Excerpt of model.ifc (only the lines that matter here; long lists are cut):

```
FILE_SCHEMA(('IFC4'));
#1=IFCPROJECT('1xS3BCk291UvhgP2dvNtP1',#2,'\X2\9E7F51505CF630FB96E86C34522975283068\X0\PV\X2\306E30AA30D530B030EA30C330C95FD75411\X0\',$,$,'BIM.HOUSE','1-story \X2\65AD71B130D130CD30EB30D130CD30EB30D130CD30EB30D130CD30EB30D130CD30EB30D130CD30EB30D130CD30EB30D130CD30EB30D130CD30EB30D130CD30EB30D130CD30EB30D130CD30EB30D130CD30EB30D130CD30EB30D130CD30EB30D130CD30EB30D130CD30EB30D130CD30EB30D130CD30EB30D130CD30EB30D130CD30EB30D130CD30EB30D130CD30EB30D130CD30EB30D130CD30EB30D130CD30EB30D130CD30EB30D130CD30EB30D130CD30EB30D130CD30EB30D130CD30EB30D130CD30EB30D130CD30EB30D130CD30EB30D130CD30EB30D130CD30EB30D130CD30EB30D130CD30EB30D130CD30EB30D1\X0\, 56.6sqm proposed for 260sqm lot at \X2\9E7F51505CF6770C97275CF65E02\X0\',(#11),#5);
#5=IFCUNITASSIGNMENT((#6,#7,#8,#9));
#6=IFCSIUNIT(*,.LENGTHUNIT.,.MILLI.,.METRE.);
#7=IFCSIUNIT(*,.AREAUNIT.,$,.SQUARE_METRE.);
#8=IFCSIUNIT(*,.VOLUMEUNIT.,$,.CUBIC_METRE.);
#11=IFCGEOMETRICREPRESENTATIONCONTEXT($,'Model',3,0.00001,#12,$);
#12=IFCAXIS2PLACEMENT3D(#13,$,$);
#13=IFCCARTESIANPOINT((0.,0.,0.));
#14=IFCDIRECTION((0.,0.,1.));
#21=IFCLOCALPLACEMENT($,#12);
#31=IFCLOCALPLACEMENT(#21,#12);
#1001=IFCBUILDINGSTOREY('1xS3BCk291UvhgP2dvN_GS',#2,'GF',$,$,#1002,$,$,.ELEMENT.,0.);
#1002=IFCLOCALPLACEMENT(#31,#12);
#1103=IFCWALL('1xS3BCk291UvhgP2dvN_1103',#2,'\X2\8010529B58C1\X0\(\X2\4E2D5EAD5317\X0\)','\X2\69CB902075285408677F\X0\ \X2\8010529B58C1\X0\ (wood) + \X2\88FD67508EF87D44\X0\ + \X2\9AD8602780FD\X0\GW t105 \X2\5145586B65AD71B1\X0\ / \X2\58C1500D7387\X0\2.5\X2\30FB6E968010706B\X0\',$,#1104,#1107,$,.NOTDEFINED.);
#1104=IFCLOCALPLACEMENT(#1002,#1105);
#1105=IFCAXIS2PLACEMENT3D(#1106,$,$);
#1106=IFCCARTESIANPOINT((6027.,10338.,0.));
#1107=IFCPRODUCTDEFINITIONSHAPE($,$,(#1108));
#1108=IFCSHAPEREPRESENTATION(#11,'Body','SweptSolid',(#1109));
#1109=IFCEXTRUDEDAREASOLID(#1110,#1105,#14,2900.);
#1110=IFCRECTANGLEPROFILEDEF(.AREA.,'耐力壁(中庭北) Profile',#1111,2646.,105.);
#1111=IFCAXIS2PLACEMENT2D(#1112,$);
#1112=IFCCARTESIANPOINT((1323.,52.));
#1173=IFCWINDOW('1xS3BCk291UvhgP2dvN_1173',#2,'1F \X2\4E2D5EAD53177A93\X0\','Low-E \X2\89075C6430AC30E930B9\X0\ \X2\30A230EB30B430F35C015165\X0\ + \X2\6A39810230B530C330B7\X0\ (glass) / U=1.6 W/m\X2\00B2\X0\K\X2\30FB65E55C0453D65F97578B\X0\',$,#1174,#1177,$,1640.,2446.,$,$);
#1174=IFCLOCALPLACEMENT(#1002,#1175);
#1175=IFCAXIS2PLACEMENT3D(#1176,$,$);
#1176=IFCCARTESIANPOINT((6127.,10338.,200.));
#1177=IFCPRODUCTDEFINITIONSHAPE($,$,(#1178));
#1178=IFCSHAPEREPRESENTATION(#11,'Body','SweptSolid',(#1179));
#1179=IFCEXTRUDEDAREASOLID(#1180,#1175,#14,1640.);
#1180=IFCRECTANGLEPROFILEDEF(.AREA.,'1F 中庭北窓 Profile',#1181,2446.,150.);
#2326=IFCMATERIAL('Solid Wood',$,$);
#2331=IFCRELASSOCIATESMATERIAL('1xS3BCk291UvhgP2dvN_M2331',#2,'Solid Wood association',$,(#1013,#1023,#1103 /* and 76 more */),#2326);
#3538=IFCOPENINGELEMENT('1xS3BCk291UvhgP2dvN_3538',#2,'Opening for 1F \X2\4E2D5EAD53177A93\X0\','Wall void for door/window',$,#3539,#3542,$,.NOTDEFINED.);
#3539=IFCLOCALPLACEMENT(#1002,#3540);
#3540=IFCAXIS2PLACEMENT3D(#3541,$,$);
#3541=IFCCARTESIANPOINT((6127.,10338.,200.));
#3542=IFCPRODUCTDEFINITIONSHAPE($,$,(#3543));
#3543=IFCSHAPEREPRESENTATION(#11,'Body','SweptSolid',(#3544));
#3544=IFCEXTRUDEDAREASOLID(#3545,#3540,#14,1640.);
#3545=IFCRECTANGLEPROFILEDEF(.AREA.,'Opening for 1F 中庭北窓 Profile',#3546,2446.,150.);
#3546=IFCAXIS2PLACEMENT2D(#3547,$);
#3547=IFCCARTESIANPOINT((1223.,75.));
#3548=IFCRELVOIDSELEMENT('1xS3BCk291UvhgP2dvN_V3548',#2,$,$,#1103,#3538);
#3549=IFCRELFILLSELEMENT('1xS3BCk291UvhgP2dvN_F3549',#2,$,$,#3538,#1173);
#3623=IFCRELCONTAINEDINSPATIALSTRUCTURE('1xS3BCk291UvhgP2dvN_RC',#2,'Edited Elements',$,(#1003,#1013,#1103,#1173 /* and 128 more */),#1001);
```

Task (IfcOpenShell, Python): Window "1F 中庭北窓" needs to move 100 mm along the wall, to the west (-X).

```python
import ifcopenshell
import ifcopenshell.api.geometry
import ifcopenshell.util.placement
import ifcopenshell.util.unit

model = ifcopenshell.open("model.ifc")
unit_scale = ifcopenshell.util.unit.calculate_unit_scale(model)

window = model.by_guid("1xS3BCk291UvhgP2dvN_1173")
opening = window.FillsVoids[0].RelatingOpeningElement
wall = opening.VoidsElements[0].RelatingBuildingElement

wall_matrix = ifcopenshell.util.placement.get_local_placement(wall.ObjectPlacement)
shift = wall_matrix[:3, 0] * -0.1 / unit_scale
before = ifcopenshell.util.placement.get_local_placement(window.ObjectPlacement)[:3, 3].copy()

# The window is not placed relative to its opening, so move both.
for product in (opening, window):
    matrix = ifcopenshell.util.placement.get_local_placement(product.ObjectPlacement)
    matrix[:3, 3] += shift
    ifcopenshell.api.geometry.edit_object_placement(model, product=product, matrix=matrix, is_si=False)

after = ifcopenshell.util.placement.get_local_placement(window.ObjectPlacement)[:3, 3]
print("window moved by", (after - before).round(3) + 0.0)

model.write("model_rev.ifc")
```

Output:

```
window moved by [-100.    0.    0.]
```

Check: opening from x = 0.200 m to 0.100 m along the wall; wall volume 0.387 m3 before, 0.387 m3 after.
